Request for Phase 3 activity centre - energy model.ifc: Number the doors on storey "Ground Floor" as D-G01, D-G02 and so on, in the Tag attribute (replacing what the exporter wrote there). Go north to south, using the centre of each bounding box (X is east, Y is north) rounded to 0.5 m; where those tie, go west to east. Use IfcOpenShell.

First a look at what the model holds.

```python
import ifcopenshell
import ifcopenshell.util.element
import ifcopenshell.util.placement

model = ifcopenshell.open("Phase 3 activity centre - energy model.ifc")
print(model.schema)
storey = next(s for s in model.by_type("IfcBuildingStorey") if s.Name == "Ground Floor")
doors = [e for e in ifcopenshell.util.element.get_decomposition(storey) if e.is_a("IfcDoor")]
for e in sorted(doors, key=lambda e: e.id()):
    origin = ifcopenshell.util.placement.get_local_placement(e.ObjectPlacement)[:3, 3]
    print(e.id(), e.Tag, e.Name, origin.round(2) + 0.0, sep=" | ")
```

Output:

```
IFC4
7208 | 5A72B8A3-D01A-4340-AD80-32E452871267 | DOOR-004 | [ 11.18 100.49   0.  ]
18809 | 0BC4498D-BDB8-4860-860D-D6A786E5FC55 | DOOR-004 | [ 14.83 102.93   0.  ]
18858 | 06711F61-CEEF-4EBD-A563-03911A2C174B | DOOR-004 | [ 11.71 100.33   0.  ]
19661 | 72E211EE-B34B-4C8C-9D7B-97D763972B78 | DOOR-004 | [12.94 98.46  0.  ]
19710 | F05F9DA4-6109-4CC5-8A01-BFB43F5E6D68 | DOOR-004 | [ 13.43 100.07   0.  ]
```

```python
import ifcopenshell
import ifcopenshell.geom
import ifcopenshell.util.element
import ifcopenshell.util.shape

model = ifcopenshell.open("Phase 3 activity centre - energy model.ifc")
settings = ifcopenshell.geom.settings()
settings.set("use-world-coords", True)


def centre(element):
    shape = ifcopenshell.geom.create_shape(settings, element)
    return ifcopenshell.util.shape.get_bbox_centroid(shape.geometry)


storey = next(s for s in model.by_type("IfcBuildingStorey") if s.Name == "Ground Floor")
doors = [e for e in ifcopenshell.util.element.get_decomposition(storey) if e.is_a("IfcDoor")]

# Insertion points can sit at a corner or the storey origin, so sort by the geometry (in metres).
centres = {e: centre(e) for e in doors}
doors.sort(key=lambda e: (-round(centres[e][1] / 0.5), centres[e][0]))

for i, e in enumerate(doors, start=1):
    number = f"D-G{i:02d}"
    e.Tag = number
    print(e.id(), number)

model.write("Phase 3 activity centre - energy model_rev.ifc")
```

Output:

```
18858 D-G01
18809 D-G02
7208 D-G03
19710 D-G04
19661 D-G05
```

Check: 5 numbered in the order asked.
